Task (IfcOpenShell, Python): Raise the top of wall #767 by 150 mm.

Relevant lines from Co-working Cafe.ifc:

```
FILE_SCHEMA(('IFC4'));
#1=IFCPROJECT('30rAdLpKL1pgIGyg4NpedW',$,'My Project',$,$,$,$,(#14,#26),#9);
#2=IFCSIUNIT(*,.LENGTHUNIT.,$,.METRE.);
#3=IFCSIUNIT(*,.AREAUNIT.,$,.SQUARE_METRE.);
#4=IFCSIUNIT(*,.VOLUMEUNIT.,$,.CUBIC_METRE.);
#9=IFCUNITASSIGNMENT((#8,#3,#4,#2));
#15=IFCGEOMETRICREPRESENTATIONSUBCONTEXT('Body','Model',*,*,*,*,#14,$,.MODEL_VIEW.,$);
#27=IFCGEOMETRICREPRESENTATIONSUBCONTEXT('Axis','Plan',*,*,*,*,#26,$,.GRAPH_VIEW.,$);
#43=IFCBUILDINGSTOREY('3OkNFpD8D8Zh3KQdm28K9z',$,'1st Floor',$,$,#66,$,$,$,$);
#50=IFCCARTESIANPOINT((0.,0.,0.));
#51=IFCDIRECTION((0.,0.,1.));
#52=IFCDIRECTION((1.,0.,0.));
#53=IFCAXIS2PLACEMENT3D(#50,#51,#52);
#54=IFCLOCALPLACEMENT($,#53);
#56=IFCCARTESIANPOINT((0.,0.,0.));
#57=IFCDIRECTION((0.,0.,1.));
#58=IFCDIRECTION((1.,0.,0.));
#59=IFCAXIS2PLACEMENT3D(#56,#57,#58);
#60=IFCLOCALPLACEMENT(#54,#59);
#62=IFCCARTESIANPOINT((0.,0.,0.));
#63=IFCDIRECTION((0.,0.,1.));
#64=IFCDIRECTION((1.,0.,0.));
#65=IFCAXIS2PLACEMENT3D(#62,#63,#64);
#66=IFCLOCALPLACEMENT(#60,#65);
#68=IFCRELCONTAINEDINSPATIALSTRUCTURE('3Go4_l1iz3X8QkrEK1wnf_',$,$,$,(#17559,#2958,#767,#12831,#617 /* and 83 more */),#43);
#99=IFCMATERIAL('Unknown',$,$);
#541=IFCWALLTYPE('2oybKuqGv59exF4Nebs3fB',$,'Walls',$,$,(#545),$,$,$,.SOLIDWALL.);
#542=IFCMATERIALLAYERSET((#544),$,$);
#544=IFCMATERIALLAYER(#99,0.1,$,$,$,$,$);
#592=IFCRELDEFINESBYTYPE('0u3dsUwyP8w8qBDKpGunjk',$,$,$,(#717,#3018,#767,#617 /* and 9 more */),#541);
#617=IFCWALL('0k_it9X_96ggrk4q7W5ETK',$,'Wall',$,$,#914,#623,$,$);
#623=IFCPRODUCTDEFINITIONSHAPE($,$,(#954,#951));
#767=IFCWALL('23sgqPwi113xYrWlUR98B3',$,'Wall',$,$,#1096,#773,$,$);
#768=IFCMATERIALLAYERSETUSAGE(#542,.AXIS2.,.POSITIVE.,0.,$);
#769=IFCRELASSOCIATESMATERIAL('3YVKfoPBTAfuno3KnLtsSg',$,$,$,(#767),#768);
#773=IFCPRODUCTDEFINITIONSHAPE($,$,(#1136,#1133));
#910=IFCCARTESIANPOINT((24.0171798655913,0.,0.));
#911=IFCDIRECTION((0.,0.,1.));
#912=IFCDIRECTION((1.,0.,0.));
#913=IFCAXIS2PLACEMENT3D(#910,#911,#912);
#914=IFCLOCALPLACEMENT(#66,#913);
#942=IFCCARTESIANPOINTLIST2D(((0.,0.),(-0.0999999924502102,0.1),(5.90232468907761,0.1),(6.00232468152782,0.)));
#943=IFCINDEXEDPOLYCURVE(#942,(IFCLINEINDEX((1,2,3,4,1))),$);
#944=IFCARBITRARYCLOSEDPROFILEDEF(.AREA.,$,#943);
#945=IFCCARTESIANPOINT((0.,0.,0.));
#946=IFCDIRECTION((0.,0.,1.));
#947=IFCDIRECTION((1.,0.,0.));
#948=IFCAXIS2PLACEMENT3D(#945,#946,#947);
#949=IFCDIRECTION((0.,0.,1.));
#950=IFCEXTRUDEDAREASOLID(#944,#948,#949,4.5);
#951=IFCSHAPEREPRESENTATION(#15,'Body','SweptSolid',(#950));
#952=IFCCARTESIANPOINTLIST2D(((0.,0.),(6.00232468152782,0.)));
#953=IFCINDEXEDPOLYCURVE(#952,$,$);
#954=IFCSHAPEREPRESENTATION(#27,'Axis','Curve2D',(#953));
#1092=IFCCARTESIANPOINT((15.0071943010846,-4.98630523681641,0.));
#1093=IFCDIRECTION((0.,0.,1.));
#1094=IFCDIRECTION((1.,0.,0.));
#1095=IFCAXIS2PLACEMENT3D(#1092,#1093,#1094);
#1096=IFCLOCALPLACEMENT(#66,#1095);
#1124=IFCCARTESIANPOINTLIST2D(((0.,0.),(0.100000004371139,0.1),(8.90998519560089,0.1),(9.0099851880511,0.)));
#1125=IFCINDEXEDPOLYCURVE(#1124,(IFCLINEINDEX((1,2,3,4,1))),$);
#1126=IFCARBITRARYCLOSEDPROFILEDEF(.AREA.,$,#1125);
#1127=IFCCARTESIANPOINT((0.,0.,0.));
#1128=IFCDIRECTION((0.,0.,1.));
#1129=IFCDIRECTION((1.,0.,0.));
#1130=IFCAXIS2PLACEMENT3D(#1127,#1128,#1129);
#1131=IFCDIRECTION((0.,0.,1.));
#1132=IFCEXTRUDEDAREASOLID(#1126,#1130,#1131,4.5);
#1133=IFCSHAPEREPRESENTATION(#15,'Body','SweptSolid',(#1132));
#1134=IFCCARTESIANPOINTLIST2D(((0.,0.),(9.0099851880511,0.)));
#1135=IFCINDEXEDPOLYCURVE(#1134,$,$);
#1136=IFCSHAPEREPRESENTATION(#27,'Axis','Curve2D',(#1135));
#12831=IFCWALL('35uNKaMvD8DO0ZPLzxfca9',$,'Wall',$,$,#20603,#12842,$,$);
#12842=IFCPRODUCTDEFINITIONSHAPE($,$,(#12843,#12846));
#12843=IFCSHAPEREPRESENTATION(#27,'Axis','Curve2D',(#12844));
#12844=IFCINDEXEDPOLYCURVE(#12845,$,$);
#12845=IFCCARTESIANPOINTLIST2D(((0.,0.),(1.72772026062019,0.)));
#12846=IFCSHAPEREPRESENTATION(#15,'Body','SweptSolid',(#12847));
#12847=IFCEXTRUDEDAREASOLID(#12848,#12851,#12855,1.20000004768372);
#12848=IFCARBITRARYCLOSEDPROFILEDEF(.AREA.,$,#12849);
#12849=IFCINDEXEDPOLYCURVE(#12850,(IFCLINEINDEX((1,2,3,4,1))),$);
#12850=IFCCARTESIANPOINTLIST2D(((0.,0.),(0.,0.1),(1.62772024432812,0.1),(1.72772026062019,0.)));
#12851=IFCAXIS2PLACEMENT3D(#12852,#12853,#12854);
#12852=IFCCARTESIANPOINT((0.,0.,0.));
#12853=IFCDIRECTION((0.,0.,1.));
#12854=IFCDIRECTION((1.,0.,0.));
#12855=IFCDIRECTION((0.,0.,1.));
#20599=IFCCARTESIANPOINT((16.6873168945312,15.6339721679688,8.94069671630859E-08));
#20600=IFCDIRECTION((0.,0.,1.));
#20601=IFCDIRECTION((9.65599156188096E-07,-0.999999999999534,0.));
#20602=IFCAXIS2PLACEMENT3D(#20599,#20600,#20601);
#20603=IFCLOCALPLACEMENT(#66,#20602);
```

```python
import ifcopenshell
import ifcopenshell.geom
import ifcopenshell.util.representation
import ifcopenshell.util.shape
import ifcopenshell.util.unit

model = ifcopenshell.open("Co-working Cafe.ifc")
unit_scale = ifcopenshell.util.unit.calculate_unit_scale(model)
settings = ifcopenshell.geom.settings()


def volume(element):
    """Net volume in cubic metres, openings subtracted."""
    shape = ifcopenshell.geom.create_shape(settings, element)
    return ifcopenshell.util.shape.get_volume(shape.geometry)


wall = model.by_guid("23sgqPwi113xYrWlUR98B3")
before = volume(wall)

body = ifcopenshell.util.representation.get_representation(wall, "Model", "Body")
solid = body.Items[0]
old_height = solid.Depth
solid.Depth += 0.15 / unit_scale
after = volume(wall)

print(f"height {old_height:g} -> {solid.Depth:g}, volume {before:.3f} -> {after:.3f} m3")

model.write("Co-working Cafe_v2.ifc")
```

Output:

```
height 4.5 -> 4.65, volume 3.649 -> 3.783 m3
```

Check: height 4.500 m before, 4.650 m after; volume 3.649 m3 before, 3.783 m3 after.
